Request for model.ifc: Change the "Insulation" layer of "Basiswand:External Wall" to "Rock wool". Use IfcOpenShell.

First a look at what the model holds.

```python
import ifcopenshell
import ifcopenshell.util.element

model = ifcopenshell.open("model.ifc")
print(model.schema)
for layer_set in model.by_type("IfcMaterialLayerSet"):
    if layer_set.LayerSetName == "Basiswand:External Wall":
        for layer in layer_set.MaterialLayers:
            print(layer.id(), layer.Material and layer.Material.Name, layer.LayerThickness, sep=" | ")
        print(len(ifcopenshell.util.element.get_elements_by_material(model, layer_set)), "elements and types use it")
print(sorted(m.Name for m in model.by_type("IfcMaterial") if m.Name)[:60])
```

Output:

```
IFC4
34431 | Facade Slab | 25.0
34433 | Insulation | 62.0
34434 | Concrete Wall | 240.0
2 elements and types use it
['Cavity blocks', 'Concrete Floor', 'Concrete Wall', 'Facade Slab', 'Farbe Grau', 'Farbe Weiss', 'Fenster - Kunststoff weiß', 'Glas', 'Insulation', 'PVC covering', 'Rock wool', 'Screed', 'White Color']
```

```python
import ifcopenshell
import ifcopenshell.api.material

model = ifcopenshell.open("model.ifc")

layer_set = next(s for s in model.by_type("IfcMaterialLayerSet") if s.LayerSetName == "Basiswand:External Wall")
layer = next(l for l in layer_set.MaterialLayers if l.Material and l.Material.Name == "Insulation")
material = next(m for m in model.by_type("IfcMaterial") if m.Name == "Rock wool")

# Point this one layer at the other material; renaming the old one would change it everywhere.
ifcopenshell.api.material.edit_layer(model, layer=layer, attributes={}, material=material)

print([l.Material.Name if l.Material else None for l in layer_set.MaterialLayers])

model.write("model-out.ifc")
```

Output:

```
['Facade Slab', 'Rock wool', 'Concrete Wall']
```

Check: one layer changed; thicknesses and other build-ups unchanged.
